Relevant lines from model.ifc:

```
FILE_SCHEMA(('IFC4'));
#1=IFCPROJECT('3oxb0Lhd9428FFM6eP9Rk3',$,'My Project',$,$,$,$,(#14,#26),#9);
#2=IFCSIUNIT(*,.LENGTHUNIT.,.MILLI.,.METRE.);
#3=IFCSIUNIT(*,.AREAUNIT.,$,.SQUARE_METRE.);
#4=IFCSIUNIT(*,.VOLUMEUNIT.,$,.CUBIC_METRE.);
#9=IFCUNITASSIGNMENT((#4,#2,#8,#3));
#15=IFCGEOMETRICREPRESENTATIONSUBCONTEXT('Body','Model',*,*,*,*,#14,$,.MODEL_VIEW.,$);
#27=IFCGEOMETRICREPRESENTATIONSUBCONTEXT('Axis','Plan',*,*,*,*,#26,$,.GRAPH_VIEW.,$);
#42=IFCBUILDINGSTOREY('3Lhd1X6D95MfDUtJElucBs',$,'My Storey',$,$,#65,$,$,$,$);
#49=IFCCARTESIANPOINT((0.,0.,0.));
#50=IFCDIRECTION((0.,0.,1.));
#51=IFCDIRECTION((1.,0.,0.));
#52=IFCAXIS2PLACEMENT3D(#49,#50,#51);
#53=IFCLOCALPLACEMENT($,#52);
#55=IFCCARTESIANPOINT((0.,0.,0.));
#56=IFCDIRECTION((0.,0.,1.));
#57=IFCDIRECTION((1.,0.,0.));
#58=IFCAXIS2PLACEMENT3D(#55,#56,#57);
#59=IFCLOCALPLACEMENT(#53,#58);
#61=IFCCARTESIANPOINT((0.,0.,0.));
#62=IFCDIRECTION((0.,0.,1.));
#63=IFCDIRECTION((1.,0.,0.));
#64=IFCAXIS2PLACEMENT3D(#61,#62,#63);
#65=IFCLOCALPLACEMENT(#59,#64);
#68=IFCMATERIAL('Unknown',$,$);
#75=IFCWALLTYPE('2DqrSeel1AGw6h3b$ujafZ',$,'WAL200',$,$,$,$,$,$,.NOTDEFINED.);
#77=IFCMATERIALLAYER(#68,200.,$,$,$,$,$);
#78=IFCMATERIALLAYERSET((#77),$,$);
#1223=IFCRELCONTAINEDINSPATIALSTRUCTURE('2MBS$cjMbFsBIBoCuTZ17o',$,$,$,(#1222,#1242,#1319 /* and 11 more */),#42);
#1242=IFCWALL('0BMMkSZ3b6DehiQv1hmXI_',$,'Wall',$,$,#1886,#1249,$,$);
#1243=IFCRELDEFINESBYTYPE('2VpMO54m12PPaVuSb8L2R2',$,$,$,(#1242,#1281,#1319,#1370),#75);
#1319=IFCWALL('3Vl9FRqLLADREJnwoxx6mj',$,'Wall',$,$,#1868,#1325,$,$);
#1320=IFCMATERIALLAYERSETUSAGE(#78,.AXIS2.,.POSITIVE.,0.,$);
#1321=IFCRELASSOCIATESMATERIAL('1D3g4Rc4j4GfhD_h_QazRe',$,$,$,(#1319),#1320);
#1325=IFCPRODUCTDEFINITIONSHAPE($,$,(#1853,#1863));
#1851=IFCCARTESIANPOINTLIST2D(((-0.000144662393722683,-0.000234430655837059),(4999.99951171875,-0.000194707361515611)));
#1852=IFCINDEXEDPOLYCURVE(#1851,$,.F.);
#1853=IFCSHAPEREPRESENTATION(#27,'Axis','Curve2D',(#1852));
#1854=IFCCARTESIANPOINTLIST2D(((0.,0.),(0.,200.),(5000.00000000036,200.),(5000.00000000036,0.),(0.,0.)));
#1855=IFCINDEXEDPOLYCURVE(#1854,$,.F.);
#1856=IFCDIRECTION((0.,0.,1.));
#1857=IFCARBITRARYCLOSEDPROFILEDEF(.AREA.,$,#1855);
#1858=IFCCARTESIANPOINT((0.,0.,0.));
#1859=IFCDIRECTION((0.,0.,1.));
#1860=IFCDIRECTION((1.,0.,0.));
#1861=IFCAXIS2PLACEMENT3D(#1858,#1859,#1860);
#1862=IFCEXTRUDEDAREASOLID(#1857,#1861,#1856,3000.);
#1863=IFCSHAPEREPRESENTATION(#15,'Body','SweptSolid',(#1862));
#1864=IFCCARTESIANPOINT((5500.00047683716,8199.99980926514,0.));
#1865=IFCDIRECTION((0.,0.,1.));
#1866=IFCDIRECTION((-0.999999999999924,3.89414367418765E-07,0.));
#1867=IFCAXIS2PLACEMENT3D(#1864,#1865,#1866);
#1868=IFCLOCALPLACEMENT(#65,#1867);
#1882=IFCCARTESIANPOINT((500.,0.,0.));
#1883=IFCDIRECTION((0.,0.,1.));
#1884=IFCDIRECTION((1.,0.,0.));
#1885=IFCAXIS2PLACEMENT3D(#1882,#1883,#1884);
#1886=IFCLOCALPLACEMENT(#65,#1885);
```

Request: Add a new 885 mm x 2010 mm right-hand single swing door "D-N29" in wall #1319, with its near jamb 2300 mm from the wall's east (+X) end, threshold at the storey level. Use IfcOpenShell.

```python
import numpy as np
import ifcopenshell
import ifcopenshell.api.feature
import ifcopenshell.api.geometry
import ifcopenshell.api.root
import ifcopenshell.api.spatial
import ifcopenshell.geom
import ifcopenshell.util.element
import ifcopenshell.util.placement
import ifcopenshell.util.representation
import ifcopenshell.util.shape
import ifcopenshell.util.unit

model = ifcopenshell.open("model.ifc")
unit_scale = ifcopenshell.util.unit.calculate_unit_scale(model)
settings = ifcopenshell.geom.settings()


def volume(element):
    """Net volume in cubic metres, openings subtracted."""
    shape = ifcopenshell.geom.create_shape(settings, element)
    return ifcopenshell.util.shape.get_volume(shape.geometry)


wall = model.by_guid("3Vl9FRqLLADREJnwoxx6mj")
storey = ifcopenshell.util.element.get_container(wall, ifc_class="IfcBuildingStorey")
context = ifcopenshell.util.representation.get_context(model, "Model", "Body", "MODEL_VIEW")
before = volume(wall)

width, height, from_end, sill = 0.885, 2.01, 2.3, 0.0  # metres

# The wall runs along its own X axis, and the end named is its -X end.
wall_shape = ifcopenshell.geom.create_shape(settings, wall)
x, y, z = ifcopenshell.util.shape.get_vertices(wall_shape.geometry).T
start = x.min() + from_end
face, thickness = float(y.min()), float(y.max() - y.min())
wall_matrix = ifcopenshell.util.placement.get_local_placement(wall.ObjectPlacement)
level = ifcopenshell.util.placement.get_local_placement(storey.ObjectPlacement)[2, 3]


def in_wall(x, y):
    """Placement at x, y metres in the wall's axes, at sill height."""
    matrix = wall_matrix.copy()
    matrix[:, 3] = wall_matrix @ np.array([x / unit_scale, y / unit_scale, 0.0, 1.0])
    matrix[2, 3] = level + sill / unit_scale
    return matrix


# Opening: a box that overshoots both wall faces by 50 mm.
opening = ifcopenshell.api.root.create_entity(model, ifc_class="IfcOpeningElement", predefined_type="OPENING")
box = ifcopenshell.api.geometry.add_wall_representation(
    model, context=context, length=width, height=height, thickness=thickness + 0.1
)
ifcopenshell.api.geometry.assign_representation(model, product=opening, representation=box)
ifcopenshell.api.geometry.edit_object_placement(model, product=opening, matrix=in_wall(start, face - 0.05), is_si=False)
ifcopenshell.api.feature.add_feature(model, feature=opening, element=wall)

door = ifcopenshell.api.root.create_entity(model, ifc_class="IfcDoor", name="D-N29", predefined_type="DOOR")
door.OverallWidth, door.OverallHeight = width / unit_scale, height / unit_scale
door.OperationType = "SINGLE_SWING_RIGHT"
body = ifcopenshell.api.geometry.add_door_representation(
    model,
    context=context,
    overall_width=door.OverallWidth,
    overall_height=door.OverallHeight,
    operation_type="SINGLE_SWING_RIGHT",
    lining_properties={"LiningDepth": thickness / unit_scale, "ThresholdDepth": thickness / unit_scale},
)
ifcopenshell.api.geometry.assign_representation(model, product=door, representation=body)
ifcopenshell.api.spatial.assign_container(model, products=[door], relating_structure=storey)
ifcopenshell.api.feature.add_filling(model, opening=opening, element=door)

# The lining spans the wall, so the door starts at the wall face.
ifcopenshell.api.geometry.edit_object_placement(model, product=door, matrix=in_wall(start, face), is_si=False)

after = volume(wall)

print(f"wall volume {before:.3f} -> {after:.3f} m3")

model.write("model_v2.ifc")
```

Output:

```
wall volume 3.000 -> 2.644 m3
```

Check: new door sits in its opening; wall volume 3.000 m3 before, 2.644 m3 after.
